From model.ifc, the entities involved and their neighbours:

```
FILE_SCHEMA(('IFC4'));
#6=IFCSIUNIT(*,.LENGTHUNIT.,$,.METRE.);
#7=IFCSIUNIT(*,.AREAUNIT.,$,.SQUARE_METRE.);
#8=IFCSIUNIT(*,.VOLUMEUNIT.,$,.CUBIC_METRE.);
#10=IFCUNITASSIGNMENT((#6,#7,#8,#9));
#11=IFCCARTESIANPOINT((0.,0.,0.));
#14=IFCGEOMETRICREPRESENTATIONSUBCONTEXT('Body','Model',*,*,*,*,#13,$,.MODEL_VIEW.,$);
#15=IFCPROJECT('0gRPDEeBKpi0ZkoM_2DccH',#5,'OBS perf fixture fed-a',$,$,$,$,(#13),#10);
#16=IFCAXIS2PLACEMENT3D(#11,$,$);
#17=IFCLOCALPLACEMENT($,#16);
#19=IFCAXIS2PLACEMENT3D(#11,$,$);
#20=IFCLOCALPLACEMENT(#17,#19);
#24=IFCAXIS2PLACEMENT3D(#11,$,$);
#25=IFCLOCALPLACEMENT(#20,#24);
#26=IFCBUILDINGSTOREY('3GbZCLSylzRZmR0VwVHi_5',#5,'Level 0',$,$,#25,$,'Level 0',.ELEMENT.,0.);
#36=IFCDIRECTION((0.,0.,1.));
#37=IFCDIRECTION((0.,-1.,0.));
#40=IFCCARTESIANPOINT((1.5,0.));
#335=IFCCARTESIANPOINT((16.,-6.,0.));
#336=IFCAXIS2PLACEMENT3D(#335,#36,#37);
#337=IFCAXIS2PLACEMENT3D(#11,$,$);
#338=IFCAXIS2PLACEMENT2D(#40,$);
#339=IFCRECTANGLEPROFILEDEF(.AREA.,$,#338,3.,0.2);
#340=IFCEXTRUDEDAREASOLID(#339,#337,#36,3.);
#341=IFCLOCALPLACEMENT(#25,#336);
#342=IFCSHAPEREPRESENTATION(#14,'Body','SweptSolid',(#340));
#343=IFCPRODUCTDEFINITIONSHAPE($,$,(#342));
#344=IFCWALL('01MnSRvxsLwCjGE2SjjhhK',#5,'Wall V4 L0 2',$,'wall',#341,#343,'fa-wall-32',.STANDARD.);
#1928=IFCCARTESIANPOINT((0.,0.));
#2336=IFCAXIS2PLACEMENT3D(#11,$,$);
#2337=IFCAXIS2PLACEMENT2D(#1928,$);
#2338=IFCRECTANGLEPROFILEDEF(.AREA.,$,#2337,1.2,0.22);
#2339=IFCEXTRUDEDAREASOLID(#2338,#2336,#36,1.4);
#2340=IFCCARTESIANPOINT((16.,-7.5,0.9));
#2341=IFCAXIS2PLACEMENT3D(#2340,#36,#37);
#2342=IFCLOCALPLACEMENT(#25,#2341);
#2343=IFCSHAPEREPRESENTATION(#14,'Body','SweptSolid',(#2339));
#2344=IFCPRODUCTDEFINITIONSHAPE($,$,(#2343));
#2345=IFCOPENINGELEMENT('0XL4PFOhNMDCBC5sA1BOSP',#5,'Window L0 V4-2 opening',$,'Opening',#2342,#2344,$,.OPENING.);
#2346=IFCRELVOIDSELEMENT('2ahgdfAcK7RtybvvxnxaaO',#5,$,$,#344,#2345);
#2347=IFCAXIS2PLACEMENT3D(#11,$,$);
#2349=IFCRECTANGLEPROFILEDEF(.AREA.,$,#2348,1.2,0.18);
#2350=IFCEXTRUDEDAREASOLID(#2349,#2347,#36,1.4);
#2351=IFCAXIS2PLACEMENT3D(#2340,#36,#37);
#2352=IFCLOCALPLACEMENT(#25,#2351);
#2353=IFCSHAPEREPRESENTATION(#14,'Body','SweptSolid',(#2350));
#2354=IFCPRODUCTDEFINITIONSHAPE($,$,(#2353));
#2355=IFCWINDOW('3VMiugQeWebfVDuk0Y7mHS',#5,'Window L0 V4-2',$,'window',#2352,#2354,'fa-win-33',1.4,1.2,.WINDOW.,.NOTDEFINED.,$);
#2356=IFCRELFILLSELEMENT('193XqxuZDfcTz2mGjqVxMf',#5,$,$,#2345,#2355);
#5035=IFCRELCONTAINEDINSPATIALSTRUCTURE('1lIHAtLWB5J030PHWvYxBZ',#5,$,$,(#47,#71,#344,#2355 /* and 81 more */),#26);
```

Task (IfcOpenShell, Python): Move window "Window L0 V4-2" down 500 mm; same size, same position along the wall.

```python
import numpy as np
import ifcopenshell
import ifcopenshell.api.geometry
import ifcopenshell.util.placement
import ifcopenshell.util.unit

model = ifcopenshell.open("model.ifc")
unit_scale = ifcopenshell.util.unit.calculate_unit_scale(model)

window = model.by_id(2355)
opening = window.FillsVoids[0].RelatingOpeningElement
dz = -0.5 / unit_scale

shift = np.array([0.0, 0.0, dz])
# The window is not placed relative to its opening, so move both.
for product in (opening, window):
    matrix = ifcopenshell.util.placement.get_local_placement(product.ObjectPlacement)
    matrix[:3, 3] += shift
    ifcopenshell.api.geometry.edit_object_placement(model, product=product, matrix=matrix, is_si=False)

print(f"moved by {dz * unit_scale:+.3f} m")

model.write("model_edited.ifc")
```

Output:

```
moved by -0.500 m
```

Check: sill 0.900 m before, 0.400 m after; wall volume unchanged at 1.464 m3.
